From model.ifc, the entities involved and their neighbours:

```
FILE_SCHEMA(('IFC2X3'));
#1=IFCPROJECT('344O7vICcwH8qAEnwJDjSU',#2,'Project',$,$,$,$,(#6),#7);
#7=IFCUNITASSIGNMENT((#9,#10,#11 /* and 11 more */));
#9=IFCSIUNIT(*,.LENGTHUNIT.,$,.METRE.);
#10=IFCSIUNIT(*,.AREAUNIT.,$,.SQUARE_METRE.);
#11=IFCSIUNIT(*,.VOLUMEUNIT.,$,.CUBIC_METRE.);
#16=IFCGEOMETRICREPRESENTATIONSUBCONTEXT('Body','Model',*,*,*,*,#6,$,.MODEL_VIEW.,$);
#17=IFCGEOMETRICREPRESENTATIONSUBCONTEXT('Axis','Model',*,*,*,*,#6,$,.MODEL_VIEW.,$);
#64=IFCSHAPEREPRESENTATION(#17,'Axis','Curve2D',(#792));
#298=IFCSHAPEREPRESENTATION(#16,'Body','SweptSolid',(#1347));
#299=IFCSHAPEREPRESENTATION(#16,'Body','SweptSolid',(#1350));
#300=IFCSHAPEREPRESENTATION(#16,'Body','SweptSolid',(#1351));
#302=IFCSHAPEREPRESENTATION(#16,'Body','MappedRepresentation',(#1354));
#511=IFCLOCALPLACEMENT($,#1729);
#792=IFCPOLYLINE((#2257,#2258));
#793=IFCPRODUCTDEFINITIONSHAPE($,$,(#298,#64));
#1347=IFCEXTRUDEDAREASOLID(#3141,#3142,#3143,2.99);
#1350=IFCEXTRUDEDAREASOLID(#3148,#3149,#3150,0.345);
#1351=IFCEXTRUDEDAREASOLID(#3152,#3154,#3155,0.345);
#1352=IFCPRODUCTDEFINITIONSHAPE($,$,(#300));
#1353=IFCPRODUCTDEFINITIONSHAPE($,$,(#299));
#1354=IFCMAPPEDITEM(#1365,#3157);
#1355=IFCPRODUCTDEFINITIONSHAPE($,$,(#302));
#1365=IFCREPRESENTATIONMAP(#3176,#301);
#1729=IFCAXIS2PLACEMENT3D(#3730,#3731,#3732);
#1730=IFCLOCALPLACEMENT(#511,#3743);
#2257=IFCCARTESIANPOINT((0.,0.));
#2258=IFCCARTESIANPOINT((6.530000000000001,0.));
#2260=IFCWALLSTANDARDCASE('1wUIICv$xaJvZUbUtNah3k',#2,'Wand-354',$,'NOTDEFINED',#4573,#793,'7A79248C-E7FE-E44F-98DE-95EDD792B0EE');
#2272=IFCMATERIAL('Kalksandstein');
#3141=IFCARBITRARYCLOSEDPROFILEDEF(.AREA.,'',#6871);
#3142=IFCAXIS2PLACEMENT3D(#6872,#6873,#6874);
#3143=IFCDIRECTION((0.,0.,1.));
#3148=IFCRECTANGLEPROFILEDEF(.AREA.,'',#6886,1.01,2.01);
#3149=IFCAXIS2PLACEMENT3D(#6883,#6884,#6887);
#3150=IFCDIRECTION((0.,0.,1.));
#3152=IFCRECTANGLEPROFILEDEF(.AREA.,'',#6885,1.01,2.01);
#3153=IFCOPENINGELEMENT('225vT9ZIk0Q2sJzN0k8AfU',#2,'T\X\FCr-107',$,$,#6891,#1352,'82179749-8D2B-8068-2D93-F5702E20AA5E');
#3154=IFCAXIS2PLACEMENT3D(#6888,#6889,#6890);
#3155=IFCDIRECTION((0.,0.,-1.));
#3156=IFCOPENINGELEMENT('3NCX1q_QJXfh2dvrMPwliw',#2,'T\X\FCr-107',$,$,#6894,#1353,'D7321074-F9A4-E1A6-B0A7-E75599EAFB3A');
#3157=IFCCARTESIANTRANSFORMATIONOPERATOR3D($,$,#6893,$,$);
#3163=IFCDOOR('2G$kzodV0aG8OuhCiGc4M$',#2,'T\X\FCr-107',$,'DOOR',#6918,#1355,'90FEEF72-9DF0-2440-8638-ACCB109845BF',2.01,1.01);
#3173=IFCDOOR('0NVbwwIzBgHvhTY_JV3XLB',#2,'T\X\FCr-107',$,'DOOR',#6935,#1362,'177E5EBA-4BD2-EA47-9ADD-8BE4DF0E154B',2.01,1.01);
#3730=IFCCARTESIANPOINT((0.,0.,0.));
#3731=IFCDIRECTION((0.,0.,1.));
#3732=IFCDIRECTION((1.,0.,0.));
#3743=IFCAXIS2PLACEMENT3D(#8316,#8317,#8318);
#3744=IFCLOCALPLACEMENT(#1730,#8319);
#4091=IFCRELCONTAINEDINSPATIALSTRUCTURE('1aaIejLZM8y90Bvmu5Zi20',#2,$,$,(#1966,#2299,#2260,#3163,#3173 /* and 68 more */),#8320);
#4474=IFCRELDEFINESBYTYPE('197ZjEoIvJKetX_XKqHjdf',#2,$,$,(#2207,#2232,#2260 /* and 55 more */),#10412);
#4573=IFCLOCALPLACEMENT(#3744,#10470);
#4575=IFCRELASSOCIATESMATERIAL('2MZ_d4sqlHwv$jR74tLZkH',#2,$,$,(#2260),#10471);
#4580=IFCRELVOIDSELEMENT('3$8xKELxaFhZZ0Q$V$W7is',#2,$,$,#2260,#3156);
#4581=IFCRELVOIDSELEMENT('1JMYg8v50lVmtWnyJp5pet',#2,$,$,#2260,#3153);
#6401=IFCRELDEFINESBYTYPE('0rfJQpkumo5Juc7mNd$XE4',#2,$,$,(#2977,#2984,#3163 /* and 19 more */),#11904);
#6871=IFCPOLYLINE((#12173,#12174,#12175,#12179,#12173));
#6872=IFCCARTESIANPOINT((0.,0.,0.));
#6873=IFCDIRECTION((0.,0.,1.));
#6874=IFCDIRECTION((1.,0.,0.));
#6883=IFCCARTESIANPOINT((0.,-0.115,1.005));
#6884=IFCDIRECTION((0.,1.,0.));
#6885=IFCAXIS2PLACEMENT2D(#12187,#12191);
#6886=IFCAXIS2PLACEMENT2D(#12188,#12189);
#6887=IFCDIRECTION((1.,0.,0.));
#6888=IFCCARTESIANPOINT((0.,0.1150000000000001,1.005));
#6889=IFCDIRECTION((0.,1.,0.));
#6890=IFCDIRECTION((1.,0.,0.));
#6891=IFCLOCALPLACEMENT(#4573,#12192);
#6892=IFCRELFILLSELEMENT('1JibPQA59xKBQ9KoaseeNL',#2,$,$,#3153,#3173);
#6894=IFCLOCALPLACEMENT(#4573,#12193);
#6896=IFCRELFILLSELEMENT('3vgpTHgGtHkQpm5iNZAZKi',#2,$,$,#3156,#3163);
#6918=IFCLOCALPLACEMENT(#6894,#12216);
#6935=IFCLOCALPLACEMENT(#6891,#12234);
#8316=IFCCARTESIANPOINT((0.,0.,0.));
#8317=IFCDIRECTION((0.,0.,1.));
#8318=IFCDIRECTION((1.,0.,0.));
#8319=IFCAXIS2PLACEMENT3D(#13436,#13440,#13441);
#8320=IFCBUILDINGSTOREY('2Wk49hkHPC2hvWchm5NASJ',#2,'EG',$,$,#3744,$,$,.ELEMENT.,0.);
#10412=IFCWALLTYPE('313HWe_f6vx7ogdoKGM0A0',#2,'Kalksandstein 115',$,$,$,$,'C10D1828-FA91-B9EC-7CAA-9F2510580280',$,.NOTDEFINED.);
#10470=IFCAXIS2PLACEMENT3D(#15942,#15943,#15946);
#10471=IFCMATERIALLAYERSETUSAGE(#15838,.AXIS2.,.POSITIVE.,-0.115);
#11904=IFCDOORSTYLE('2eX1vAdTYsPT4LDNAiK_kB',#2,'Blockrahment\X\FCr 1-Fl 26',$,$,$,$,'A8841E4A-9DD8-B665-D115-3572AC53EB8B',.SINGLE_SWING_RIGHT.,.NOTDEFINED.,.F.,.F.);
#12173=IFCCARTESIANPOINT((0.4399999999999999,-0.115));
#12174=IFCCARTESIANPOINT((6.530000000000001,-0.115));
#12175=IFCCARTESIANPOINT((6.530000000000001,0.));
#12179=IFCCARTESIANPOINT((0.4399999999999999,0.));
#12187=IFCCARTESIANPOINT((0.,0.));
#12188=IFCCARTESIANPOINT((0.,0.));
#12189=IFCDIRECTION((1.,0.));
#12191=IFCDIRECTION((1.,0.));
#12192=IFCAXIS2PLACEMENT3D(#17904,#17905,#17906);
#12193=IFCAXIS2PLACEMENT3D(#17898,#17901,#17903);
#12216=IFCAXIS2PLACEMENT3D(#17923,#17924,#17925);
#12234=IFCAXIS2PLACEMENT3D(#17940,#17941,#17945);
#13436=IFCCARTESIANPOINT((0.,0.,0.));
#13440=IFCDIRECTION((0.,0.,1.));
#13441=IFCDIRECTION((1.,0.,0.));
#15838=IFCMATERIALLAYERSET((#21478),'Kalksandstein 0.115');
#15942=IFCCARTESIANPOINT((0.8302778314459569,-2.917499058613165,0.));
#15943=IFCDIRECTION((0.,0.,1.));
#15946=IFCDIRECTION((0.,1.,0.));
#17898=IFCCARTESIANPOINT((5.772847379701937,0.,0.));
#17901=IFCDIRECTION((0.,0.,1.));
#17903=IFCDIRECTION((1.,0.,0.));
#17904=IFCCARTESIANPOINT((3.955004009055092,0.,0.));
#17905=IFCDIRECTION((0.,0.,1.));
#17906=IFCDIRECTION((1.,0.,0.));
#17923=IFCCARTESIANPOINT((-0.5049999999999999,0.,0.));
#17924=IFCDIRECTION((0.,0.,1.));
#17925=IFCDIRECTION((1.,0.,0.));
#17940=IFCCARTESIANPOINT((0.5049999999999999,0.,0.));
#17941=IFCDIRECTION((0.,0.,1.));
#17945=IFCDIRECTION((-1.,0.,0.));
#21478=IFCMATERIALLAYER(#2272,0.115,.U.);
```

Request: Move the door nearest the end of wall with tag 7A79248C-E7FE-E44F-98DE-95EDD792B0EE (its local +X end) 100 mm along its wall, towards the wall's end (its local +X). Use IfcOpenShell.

```python
import ifcopenshell
import ifcopenshell.api.geometry
import ifcopenshell.util.placement
import ifcopenshell.util.unit

model = ifcopenshell.open("model.ifc")
unit_scale = ifcopenshell.util.unit.calculate_unit_scale(model)

door = model.by_guid("2G$kzodV0aG8OuhCiGc4M$")
opening = door.FillsVoids[0].RelatingOpeningElement
wall = opening.VoidsElements[0].RelatingBuildingElement

wall_matrix = ifcopenshell.util.placement.get_local_placement(wall.ObjectPlacement)
shift = wall_matrix[:3, 0] * 0.1 / unit_scale
before = ifcopenshell.util.placement.get_local_placement(door.ObjectPlacement)[:3, 3].copy()

# The door is placed relative to its opening, so it follows when the opening moves.
matrix = ifcopenshell.util.placement.get_local_placement(opening.ObjectPlacement)
matrix[:3, 3] += shift
ifcopenshell.api.geometry.edit_object_placement(
    model, product=opening, matrix=matrix, is_si=False, should_transform_children=True
)

after = ifcopenshell.util.placement.get_local_placement(door.ObjectPlacement)[:3, 3]
print("door moved by", (after - before).round(3) + 0.0)

model.write("model_v2.ifc")
```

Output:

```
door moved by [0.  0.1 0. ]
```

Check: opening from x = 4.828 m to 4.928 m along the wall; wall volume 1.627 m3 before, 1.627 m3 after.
